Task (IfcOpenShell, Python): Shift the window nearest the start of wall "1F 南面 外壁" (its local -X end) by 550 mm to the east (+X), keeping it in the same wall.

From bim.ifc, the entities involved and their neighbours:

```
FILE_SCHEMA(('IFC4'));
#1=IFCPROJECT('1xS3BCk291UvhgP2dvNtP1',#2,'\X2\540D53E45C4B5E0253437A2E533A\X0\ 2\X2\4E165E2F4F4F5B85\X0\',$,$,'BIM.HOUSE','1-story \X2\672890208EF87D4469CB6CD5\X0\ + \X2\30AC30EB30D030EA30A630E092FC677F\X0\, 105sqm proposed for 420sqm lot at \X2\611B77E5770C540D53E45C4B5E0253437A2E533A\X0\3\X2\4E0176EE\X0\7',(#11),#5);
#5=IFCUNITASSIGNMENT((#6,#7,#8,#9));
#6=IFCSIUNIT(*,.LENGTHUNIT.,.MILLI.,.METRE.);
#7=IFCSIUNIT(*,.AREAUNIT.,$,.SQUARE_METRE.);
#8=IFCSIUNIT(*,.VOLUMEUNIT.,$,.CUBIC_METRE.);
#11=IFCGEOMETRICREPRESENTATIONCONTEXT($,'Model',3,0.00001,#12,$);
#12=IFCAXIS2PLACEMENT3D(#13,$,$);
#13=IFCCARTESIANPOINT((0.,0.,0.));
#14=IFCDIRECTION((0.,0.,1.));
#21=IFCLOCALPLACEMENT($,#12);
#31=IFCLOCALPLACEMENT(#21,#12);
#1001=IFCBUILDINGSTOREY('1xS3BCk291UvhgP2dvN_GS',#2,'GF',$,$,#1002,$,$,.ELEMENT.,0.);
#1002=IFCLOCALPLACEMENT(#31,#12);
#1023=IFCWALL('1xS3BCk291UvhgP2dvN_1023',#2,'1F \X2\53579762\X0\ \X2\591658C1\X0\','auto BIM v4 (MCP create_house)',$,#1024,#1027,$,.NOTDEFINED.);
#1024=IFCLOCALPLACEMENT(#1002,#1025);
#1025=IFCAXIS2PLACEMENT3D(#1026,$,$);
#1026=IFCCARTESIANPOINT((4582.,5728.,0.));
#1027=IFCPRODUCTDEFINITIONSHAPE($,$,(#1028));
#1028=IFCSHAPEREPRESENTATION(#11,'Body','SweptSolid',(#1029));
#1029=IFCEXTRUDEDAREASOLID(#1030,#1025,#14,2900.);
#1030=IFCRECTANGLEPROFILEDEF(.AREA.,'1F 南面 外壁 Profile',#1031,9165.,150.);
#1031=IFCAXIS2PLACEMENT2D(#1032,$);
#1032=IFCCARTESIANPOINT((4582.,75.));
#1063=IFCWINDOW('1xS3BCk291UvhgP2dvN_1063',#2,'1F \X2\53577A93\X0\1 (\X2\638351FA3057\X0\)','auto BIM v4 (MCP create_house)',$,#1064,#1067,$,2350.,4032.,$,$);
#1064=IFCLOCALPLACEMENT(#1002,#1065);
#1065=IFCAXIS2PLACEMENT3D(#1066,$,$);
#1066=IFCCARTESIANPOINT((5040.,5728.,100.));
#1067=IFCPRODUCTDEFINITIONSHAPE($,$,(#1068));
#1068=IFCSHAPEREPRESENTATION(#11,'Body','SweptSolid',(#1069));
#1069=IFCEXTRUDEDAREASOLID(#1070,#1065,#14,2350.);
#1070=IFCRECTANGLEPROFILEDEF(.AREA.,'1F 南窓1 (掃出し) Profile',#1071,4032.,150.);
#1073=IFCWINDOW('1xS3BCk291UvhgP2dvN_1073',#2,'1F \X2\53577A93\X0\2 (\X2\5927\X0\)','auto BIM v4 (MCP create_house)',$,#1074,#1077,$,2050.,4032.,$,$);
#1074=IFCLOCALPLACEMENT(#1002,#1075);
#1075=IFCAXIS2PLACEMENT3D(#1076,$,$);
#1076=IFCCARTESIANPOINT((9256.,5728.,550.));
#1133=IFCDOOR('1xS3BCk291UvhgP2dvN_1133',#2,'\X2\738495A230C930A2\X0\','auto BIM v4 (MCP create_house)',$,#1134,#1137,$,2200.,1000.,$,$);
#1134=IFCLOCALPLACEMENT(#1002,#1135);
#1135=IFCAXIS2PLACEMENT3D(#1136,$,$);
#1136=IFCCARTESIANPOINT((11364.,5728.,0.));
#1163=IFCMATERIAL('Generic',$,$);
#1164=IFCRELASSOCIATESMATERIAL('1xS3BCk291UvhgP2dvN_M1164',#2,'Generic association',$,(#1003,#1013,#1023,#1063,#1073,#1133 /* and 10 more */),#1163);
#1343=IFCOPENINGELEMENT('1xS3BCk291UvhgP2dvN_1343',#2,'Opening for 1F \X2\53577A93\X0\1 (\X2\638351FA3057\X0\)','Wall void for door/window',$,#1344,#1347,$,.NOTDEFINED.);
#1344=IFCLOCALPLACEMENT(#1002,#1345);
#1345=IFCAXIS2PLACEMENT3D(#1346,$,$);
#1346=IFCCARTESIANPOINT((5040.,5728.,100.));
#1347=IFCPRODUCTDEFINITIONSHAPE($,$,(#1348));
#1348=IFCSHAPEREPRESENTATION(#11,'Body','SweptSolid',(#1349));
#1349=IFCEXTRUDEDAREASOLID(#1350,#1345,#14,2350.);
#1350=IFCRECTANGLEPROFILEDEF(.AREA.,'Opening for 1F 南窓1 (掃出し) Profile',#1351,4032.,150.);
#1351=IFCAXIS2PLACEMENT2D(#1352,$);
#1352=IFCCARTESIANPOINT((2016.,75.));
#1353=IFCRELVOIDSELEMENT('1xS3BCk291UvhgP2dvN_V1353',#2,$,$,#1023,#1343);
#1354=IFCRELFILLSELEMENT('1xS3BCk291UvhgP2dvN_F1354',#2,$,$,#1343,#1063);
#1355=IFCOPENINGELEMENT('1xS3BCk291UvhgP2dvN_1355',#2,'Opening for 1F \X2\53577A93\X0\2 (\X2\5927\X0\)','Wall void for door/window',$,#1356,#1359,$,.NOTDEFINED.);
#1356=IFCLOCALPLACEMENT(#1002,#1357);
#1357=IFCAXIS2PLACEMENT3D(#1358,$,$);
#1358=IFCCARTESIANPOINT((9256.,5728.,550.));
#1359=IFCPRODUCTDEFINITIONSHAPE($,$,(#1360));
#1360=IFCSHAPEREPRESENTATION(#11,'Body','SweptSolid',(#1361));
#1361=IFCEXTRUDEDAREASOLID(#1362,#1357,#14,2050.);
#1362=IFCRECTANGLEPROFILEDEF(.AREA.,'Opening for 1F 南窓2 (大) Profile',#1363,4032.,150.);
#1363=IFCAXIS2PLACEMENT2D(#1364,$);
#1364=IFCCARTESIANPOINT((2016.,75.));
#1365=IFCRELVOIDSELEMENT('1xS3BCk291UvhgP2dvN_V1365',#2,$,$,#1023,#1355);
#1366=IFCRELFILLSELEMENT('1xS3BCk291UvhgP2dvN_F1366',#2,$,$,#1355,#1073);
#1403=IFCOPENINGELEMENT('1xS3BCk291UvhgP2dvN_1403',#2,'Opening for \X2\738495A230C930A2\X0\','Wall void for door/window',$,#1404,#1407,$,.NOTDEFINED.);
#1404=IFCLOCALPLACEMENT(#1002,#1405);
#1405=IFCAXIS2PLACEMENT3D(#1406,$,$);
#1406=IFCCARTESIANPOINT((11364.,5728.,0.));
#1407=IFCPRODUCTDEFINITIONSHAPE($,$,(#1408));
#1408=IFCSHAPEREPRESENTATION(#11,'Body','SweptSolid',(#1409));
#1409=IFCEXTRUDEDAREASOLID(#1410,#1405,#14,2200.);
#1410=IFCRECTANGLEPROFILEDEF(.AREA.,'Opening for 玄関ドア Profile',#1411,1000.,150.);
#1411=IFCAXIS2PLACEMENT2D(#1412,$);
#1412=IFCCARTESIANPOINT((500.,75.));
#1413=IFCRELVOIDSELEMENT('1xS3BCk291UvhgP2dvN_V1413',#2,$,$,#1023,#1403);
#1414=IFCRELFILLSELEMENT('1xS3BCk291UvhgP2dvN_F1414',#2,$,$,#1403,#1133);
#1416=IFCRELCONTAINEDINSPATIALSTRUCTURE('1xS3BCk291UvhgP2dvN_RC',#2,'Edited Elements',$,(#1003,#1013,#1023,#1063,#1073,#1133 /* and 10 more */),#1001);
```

```python
import ifcopenshell
import ifcopenshell.api.geometry
import ifcopenshell.util.placement
import ifcopenshell.util.unit

model = ifcopenshell.open("bim.ifc")
unit_scale = ifcopenshell.util.unit.calculate_unit_scale(model)

window = model.by_guid("1xS3BCk291UvhgP2dvN_1063")
opening = window.FillsVoids[0].RelatingOpeningElement
wall = opening.VoidsElements[0].RelatingBuildingElement

wall_matrix = ifcopenshell.util.placement.get_local_placement(wall.ObjectPlacement)
shift = wall_matrix[:3, 0] * 0.55 / unit_scale
before = ifcopenshell.util.placement.get_local_placement(window.ObjectPlacement)[:3, 3].copy()

# The window is not placed relative to its opening, so move both.
for product in (opening, window):
    matrix = ifcopenshell.util.placement.get_local_placement(product.ObjectPlacement)
    matrix[:3, 3] += shift
    ifcopenshell.api.geometry.edit_object_placement(model, product=product, matrix=matrix, is_si=False)

after = ifcopenshell.util.placement.get_local_placement(window.ObjectPlacement)[:3, 3]
print("window moved by", (after - before).round(3) + 0.0)

model.write("bim_v2.ifc")
```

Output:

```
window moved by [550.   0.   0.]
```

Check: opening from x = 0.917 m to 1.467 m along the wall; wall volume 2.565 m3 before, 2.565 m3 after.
